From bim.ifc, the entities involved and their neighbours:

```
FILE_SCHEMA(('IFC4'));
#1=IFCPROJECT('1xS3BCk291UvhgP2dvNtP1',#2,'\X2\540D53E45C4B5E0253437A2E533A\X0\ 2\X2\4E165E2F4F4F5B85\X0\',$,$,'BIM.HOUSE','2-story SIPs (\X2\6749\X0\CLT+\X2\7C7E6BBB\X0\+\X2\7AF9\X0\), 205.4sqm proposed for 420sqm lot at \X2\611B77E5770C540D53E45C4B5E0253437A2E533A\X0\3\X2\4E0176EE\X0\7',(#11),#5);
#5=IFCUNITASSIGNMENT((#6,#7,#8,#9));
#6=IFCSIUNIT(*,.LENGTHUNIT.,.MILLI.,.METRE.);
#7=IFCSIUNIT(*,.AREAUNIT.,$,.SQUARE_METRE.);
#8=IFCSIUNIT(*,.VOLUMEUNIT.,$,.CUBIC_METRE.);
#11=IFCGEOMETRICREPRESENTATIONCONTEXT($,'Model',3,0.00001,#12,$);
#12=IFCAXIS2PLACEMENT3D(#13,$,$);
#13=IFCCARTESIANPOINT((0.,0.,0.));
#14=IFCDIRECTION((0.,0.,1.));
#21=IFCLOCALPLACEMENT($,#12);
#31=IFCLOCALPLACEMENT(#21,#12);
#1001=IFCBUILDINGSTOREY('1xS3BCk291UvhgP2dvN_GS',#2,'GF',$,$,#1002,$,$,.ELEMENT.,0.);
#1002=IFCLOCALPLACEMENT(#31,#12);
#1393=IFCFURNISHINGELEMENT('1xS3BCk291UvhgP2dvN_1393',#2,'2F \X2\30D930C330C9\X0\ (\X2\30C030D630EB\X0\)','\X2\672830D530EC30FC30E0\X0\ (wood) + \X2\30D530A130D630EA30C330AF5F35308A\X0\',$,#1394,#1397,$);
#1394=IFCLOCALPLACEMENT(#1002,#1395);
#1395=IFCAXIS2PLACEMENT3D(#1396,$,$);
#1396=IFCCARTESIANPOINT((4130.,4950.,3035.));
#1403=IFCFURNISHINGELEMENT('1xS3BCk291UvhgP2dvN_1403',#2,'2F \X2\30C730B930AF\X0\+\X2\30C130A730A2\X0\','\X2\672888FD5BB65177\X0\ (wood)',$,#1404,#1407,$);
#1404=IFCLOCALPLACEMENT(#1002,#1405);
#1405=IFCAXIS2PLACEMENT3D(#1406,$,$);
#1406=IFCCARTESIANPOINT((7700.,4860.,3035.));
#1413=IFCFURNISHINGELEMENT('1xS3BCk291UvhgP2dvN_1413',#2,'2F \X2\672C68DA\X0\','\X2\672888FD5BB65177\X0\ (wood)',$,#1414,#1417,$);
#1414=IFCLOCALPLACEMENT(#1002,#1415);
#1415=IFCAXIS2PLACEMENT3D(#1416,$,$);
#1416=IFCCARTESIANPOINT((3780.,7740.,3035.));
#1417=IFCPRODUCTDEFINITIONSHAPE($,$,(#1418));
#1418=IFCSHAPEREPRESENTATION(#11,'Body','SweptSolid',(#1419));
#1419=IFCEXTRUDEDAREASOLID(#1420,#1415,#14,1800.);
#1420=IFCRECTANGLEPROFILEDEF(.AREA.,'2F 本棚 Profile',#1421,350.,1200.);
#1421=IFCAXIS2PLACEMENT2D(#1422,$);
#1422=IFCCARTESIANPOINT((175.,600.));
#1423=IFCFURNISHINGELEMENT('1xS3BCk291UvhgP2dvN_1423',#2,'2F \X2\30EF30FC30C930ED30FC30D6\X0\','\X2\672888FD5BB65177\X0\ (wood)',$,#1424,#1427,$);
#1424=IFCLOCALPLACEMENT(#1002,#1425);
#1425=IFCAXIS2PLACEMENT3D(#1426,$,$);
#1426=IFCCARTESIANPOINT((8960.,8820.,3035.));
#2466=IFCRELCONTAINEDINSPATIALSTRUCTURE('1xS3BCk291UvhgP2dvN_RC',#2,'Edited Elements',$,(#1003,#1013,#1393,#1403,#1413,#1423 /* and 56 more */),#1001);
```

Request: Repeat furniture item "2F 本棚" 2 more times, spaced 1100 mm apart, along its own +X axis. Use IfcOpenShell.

```python
import ifcopenshell
import ifcopenshell.api.geometry
import ifcopenshell.api.root
import ifcopenshell.util.element
import ifcopenshell.util.placement
import ifcopenshell.util.unit

model = ifcopenshell.open("bim.ifc")
unit_scale = ifcopenshell.util.unit.calculate_unit_scale(model)


def reuse_history(source, copy):
    """copy_class also copies each property set's owner history, people and application; keep the originals."""
    for rel in copy.IsDefinedBy:
        if rel.is_a("IfcRelDefinesByProperties") and (history := rel.RelatingPropertyDefinition.OwnerHistory):
            rel.RelatingPropertyDefinition.OwnerHistory = source.OwnerHistory
            ifcopenshell.util.element.remove_deep2(model, history)


source = model.by_guid("1xS3BCk291UvhgP2dvN_1413")
base = ifcopenshell.util.placement.get_local_placement(source.ObjectPlacement)
step = base[:3, 0] * 1.1 / unit_scale

for i in range(1, 3):
    copy = ifcopenshell.api.root.copy_class(model, product=source)
    copy.Representation = ifcopenshell.util.element.copy_deep(
        model, source.Representation, exclude=["IfcGeometricRepresentationContext", "IfcRepresentationMap"]
    )
    reuse_history(source, copy)
    matrix = base.copy()
    matrix[:3, 3] += i * step
    print("added at", matrix[:3, 3].round(3) + 0.0)
    ifcopenshell.api.geometry.edit_object_placement(model, product=copy, matrix=matrix, is_si=False)

model.write("bim_edited.ifc")
```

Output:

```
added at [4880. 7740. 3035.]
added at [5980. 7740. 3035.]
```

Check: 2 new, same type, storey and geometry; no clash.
